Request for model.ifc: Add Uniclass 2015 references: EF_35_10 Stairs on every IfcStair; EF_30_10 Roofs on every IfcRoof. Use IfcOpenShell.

First a look at what the model holds.

```python
import ifcopenshell

model = ifcopenshell.open("model.ifc")
print(model.schema)
print("classifications:", [c.Name for c in model.by_type("IfcClassification")])
for ifc_class in ("IfcDoor", "IfcRoof", "IfcStair", "IfcWall", "IfcWindow"):
    print(ifc_class, len(model.by_type(ifc_class)))
```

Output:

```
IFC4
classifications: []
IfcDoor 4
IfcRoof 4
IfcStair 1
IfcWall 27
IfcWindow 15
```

```python
import ifcopenshell
import ifcopenshell.api.classification

model = ifcopenshell.open("model.ifc")

system = ifcopenshell.api.classification.add_classification(model, classification="Uniclass 2015")

codes = {
    "IfcStair": ("EF_35_10", "Stairs"),
    "IfcRoof": ("EF_30_10", "Roofs"),
}
for ifc_class, (code, name) in codes.items():
    products = model.by_type(ifc_class)
    ifcopenshell.api.classification.add_reference(
        model, products=products, classification=system, identification=code, name=name
    )
    print(code, len(products))

model.write("model_updated.ifc")
```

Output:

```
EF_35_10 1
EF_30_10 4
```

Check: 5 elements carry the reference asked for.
